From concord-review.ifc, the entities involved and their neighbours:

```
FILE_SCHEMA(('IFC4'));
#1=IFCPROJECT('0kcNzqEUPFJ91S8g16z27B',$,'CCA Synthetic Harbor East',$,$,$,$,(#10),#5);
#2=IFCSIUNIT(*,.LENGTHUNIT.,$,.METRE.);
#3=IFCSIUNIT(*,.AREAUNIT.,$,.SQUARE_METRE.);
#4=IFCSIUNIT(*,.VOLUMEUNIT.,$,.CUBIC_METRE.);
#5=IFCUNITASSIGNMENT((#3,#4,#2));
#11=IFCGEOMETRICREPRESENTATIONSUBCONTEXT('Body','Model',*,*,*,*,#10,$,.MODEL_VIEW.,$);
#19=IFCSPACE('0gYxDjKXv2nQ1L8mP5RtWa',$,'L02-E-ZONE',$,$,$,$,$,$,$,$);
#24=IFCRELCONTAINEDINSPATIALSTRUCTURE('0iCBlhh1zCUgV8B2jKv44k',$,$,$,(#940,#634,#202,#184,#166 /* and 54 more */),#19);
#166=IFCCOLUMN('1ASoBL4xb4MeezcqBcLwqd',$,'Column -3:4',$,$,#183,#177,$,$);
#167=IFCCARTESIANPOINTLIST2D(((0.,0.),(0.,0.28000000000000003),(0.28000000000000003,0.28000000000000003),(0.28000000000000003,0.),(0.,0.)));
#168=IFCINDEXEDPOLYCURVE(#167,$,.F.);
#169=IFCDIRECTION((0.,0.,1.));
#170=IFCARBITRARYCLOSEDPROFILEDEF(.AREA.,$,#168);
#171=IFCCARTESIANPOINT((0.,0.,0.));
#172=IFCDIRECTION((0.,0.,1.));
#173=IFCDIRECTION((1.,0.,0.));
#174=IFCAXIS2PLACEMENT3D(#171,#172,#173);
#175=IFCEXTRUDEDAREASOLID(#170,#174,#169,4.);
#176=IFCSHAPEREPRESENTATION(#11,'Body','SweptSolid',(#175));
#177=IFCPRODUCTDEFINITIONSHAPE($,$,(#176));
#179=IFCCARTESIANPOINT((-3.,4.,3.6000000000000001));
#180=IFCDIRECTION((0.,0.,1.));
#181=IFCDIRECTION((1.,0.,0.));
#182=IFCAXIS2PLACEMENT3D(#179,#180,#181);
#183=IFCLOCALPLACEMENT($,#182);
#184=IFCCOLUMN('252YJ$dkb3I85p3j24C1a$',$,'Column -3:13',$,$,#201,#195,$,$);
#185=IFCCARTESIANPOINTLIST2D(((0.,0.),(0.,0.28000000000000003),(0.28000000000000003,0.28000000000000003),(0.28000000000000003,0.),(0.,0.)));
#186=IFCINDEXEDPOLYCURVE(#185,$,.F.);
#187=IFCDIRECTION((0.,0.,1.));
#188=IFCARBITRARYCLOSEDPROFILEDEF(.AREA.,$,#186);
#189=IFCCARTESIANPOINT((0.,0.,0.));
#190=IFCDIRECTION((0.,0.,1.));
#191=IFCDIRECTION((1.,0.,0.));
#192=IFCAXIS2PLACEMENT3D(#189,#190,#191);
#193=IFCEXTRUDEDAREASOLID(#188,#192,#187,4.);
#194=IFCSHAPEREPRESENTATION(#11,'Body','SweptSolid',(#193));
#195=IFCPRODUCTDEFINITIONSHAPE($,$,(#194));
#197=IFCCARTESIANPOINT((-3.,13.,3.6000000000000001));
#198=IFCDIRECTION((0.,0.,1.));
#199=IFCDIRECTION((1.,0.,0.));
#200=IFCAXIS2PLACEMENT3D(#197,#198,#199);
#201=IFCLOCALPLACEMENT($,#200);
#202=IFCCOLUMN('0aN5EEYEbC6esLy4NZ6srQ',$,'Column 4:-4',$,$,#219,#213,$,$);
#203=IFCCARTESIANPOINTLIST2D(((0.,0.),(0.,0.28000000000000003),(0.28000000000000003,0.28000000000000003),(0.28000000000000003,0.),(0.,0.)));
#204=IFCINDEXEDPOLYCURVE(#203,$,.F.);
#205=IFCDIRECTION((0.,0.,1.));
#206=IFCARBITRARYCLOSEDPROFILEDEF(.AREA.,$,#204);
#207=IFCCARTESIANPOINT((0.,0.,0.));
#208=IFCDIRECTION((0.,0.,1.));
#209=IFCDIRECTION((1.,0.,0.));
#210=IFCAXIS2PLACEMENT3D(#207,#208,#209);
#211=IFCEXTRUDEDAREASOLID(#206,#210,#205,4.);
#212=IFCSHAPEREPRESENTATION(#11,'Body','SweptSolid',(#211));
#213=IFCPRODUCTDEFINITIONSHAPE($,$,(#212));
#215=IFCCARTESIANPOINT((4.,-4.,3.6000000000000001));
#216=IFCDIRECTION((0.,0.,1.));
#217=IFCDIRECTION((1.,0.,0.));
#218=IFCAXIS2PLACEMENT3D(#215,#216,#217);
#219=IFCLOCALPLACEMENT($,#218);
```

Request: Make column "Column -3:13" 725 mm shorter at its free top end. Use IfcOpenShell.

```python
import ifcopenshell
import ifcopenshell.util.representation

model = ifcopenshell.open("concord-review.ifc")

member = model.by_id(184)
change = -0.725

# The extrusion runs towards the end named, so only its depth changes.
body = ifcopenshell.util.representation.get_representation(member, "Model", "Body")
solid = body.Items[0]
old_length = solid.Depth
solid.Depth += change

print(f"length {old_length:g} -> {solid.Depth:g}")

model.write("concord-review_edited.ifc")
```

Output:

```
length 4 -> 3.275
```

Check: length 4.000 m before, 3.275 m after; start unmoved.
